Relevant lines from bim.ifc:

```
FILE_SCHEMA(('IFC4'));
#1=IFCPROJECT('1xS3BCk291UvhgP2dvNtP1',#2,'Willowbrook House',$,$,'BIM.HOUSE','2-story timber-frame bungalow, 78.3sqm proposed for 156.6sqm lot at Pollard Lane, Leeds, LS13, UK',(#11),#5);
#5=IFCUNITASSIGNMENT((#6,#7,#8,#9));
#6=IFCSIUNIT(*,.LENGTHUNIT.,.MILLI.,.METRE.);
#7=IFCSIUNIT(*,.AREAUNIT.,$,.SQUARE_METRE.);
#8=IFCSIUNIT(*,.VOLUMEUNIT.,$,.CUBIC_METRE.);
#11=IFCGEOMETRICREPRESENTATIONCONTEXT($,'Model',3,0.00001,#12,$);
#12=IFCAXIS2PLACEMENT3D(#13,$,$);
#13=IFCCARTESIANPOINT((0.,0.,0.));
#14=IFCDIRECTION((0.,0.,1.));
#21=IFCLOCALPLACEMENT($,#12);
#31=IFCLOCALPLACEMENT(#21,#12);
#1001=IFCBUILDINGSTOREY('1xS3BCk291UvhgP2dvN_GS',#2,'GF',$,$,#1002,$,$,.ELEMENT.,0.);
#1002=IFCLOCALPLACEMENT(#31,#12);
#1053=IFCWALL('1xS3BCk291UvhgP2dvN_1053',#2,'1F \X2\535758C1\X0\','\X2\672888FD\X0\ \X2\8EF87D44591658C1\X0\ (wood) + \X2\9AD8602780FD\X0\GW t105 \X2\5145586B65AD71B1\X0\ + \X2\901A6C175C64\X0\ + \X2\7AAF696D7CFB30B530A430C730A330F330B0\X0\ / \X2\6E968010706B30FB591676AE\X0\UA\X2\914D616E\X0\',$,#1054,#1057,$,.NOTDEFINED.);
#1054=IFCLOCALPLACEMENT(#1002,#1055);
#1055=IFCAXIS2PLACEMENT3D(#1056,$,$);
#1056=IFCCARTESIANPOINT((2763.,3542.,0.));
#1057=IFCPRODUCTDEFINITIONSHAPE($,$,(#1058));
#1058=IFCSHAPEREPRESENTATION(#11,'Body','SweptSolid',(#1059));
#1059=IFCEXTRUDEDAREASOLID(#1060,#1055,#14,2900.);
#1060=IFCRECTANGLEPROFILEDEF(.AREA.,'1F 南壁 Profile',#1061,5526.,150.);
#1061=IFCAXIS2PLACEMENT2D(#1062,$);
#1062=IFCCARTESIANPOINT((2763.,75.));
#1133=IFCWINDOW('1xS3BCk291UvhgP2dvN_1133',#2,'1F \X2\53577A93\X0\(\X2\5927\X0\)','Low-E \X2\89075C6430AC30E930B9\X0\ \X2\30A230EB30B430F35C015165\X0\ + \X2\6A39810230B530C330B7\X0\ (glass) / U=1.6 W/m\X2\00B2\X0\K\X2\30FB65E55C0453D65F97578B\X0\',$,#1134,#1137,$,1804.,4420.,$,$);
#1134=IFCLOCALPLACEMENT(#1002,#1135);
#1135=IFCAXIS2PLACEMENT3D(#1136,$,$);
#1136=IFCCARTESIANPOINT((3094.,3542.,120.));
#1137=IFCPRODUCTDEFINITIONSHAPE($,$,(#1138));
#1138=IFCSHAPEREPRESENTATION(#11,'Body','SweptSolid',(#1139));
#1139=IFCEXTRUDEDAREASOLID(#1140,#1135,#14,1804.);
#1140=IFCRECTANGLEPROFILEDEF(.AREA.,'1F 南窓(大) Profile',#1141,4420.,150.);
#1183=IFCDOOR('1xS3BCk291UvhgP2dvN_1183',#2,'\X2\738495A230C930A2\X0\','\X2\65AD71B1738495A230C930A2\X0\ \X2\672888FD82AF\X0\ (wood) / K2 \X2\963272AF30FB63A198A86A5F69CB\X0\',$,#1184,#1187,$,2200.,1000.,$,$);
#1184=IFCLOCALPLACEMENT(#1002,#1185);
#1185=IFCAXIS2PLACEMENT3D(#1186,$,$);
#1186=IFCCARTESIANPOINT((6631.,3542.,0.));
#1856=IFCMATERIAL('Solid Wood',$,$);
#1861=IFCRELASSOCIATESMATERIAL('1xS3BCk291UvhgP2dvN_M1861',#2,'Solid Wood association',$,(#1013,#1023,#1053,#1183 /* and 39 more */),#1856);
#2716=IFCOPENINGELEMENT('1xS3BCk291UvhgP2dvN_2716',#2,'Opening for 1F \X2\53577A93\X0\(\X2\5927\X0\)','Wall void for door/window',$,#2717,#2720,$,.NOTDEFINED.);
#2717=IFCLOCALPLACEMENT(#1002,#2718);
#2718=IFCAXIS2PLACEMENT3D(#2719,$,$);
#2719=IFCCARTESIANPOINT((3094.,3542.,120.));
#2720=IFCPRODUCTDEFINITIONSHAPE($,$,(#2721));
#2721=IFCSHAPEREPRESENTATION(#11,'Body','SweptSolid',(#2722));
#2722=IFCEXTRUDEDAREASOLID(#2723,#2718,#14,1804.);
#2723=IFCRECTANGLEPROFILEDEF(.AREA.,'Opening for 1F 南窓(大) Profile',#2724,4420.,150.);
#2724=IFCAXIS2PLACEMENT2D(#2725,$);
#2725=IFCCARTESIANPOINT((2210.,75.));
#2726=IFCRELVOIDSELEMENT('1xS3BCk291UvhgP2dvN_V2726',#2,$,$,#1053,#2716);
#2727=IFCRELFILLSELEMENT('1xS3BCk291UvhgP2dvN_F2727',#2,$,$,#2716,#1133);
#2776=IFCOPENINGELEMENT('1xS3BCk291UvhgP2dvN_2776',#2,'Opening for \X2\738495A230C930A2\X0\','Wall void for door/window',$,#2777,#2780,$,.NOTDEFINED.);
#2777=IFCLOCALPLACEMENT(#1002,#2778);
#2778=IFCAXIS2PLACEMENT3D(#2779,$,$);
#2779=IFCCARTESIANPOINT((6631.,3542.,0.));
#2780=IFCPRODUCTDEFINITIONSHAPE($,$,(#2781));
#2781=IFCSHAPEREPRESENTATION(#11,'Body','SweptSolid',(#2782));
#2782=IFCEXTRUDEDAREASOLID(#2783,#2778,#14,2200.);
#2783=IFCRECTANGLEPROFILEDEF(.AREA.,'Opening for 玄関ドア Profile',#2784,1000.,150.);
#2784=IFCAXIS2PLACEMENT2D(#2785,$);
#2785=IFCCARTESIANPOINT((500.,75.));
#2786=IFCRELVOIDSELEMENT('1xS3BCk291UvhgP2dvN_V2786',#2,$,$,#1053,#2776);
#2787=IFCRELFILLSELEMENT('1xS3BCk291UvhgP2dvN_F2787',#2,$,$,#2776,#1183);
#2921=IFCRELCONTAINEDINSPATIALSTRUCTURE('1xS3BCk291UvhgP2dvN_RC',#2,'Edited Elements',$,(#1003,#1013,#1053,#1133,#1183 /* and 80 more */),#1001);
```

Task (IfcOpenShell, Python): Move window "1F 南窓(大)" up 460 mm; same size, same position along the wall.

```python
import numpy as np
import ifcopenshell
import ifcopenshell.api.geometry
import ifcopenshell.util.placement
import ifcopenshell.util.unit

model = ifcopenshell.open("bim.ifc")
unit_scale = ifcopenshell.util.unit.calculate_unit_scale(model)

window = model.by_guid("1xS3BCk291UvhgP2dvN_1133")
opening = window.FillsVoids[0].RelatingOpeningElement
dz = 0.46 / unit_scale

shift = np.array([0.0, 0.0, dz])
# The window is not placed relative to its opening, so move both.
for product in (opening, window):
    matrix = ifcopenshell.util.placement.get_local_placement(product.ObjectPlacement)
    matrix[:3, 3] += shift
    ifcopenshell.api.geometry.edit_object_placement(model, product=product, matrix=matrix, is_si=False)

print(f"moved by {dz * unit_scale:+.3f} m")

model.write("bim_updated.ifc")
```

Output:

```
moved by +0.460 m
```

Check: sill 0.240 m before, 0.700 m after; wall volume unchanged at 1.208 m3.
